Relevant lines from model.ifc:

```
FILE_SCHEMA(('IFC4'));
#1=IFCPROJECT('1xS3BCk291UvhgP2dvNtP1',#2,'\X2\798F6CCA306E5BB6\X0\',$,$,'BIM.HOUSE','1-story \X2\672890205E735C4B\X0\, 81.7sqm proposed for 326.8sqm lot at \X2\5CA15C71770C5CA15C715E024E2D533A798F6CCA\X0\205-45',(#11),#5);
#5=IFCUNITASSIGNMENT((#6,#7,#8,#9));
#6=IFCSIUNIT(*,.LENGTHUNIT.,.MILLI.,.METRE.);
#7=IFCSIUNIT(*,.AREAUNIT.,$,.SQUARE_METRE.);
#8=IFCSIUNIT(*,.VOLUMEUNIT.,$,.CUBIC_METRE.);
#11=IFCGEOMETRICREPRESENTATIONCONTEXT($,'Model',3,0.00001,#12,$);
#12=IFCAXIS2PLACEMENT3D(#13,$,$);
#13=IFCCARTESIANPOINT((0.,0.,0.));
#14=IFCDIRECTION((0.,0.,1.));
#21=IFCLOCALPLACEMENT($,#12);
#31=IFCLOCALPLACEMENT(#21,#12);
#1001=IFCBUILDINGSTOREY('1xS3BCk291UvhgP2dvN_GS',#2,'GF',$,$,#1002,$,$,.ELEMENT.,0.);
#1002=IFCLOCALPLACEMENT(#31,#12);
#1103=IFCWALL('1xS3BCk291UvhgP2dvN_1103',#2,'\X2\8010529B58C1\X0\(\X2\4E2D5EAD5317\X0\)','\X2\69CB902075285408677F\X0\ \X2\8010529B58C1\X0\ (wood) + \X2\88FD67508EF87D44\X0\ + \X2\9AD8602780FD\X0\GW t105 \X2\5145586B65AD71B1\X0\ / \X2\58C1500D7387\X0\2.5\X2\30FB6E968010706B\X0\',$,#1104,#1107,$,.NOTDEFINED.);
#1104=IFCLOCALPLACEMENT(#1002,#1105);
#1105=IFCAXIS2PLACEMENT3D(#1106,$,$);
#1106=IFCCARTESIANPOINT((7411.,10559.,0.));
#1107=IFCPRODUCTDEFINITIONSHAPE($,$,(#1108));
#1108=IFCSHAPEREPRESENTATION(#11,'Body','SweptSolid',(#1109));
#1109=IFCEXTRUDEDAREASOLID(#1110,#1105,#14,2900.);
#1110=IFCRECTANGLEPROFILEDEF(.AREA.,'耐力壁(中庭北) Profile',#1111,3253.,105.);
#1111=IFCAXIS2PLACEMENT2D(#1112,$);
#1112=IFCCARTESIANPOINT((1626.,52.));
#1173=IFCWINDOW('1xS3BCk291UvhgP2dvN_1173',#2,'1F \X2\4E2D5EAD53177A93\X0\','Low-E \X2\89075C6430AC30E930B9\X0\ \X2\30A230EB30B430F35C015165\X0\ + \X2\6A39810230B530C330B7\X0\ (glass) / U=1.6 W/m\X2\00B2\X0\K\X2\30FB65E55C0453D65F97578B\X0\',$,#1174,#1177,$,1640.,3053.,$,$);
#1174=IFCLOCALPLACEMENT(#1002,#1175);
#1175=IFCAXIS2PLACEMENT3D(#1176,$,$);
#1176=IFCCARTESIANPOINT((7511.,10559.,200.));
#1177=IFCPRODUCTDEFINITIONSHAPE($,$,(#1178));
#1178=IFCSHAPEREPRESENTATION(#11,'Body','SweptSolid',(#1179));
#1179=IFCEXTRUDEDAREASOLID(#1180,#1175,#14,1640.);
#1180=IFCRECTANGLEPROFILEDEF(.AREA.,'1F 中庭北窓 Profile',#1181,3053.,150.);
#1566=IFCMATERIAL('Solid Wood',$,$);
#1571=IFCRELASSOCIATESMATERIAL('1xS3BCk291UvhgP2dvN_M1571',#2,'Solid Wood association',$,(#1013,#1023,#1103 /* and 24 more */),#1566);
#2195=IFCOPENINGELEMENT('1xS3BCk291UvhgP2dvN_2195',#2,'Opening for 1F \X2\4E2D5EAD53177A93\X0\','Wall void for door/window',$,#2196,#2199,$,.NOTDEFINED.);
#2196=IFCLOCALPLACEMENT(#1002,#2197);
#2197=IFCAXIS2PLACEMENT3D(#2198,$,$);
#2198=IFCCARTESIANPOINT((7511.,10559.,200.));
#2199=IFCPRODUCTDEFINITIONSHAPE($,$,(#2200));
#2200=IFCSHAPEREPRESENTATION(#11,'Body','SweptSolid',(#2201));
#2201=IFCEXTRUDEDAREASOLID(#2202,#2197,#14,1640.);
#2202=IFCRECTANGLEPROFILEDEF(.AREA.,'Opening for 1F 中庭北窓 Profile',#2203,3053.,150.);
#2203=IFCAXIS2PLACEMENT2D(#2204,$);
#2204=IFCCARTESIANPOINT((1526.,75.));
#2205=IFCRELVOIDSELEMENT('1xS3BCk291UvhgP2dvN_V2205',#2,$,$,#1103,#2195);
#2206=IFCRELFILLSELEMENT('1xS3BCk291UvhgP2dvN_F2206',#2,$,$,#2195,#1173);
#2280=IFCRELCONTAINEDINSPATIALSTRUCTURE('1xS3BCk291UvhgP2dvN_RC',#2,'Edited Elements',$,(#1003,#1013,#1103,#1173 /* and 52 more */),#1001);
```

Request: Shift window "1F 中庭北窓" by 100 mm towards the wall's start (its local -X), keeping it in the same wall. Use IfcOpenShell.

```python
import ifcopenshell
import ifcopenshell.api.geometry
import ifcopenshell.util.placement
import ifcopenshell.util.unit

model = ifcopenshell.open("model.ifc")
unit_scale = ifcopenshell.util.unit.calculate_unit_scale(model)

window = model.by_id(1173)
opening = window.FillsVoids[0].RelatingOpeningElement
wall = opening.VoidsElements[0].RelatingBuildingElement

wall_matrix = ifcopenshell.util.placement.get_local_placement(wall.ObjectPlacement)
shift = wall_matrix[:3, 0] * -0.1 / unit_scale
before = ifcopenshell.util.placement.get_local_placement(window.ObjectPlacement)[:3, 3].copy()

# The window is not placed relative to its opening, so move both.
for product in (opening, window):
    matrix = ifcopenshell.util.placement.get_local_placement(product.ObjectPlacement)
    matrix[:3, 3] += shift
    ifcopenshell.api.geometry.edit_object_placement(model, product=product, matrix=matrix, is_si=False)

after = ifcopenshell.util.placement.get_local_placement(window.ObjectPlacement)[:3, 3]
print("window moved by", (after - before).round(3) + 0.0)

model.write("model-out.ifc")
```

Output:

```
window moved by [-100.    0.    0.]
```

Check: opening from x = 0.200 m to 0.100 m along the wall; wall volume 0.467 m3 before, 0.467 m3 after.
